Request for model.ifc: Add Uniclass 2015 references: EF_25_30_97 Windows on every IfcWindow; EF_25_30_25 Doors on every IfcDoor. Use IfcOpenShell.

First a look at what the model holds.

```python
import ifcopenshell

model = ifcopenshell.open("model.ifc")
print(model.schema)
print("classifications:", [c.Name for c in model.by_type("IfcClassification")])
for ifc_class in ("IfcDoor", "IfcRoof", "IfcStair", "IfcWall", "IfcWindow"):
    print(ifc_class, len(model.by_type(ifc_class)))
```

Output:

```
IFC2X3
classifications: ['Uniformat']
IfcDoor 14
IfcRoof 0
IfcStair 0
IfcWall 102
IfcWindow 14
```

```python
import ifcopenshell
import ifcopenshell.api.classification

model = ifcopenshell.open("model.ifc")

# IFC2X3 requires Source and Edition and has no link from the project to the system.
system = model.create_entity("IfcClassification", Source="NBS", Edition="2015", Name="Uniclass 2015")

codes = {
    "IfcWindow": ("EF_25_30_97", "Windows"),
    "IfcDoor": ("EF_25_30_25", "Doors"),
}
for ifc_class, (code, name) in codes.items():
    products = model.by_type(ifc_class)
    ifcopenshell.api.classification.add_reference(
        model, products=products, classification=system, identification=code, name=name
    )
    print(code, len(products))

model.write("model_edited.ifc")
```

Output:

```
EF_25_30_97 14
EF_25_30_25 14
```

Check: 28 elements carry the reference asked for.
